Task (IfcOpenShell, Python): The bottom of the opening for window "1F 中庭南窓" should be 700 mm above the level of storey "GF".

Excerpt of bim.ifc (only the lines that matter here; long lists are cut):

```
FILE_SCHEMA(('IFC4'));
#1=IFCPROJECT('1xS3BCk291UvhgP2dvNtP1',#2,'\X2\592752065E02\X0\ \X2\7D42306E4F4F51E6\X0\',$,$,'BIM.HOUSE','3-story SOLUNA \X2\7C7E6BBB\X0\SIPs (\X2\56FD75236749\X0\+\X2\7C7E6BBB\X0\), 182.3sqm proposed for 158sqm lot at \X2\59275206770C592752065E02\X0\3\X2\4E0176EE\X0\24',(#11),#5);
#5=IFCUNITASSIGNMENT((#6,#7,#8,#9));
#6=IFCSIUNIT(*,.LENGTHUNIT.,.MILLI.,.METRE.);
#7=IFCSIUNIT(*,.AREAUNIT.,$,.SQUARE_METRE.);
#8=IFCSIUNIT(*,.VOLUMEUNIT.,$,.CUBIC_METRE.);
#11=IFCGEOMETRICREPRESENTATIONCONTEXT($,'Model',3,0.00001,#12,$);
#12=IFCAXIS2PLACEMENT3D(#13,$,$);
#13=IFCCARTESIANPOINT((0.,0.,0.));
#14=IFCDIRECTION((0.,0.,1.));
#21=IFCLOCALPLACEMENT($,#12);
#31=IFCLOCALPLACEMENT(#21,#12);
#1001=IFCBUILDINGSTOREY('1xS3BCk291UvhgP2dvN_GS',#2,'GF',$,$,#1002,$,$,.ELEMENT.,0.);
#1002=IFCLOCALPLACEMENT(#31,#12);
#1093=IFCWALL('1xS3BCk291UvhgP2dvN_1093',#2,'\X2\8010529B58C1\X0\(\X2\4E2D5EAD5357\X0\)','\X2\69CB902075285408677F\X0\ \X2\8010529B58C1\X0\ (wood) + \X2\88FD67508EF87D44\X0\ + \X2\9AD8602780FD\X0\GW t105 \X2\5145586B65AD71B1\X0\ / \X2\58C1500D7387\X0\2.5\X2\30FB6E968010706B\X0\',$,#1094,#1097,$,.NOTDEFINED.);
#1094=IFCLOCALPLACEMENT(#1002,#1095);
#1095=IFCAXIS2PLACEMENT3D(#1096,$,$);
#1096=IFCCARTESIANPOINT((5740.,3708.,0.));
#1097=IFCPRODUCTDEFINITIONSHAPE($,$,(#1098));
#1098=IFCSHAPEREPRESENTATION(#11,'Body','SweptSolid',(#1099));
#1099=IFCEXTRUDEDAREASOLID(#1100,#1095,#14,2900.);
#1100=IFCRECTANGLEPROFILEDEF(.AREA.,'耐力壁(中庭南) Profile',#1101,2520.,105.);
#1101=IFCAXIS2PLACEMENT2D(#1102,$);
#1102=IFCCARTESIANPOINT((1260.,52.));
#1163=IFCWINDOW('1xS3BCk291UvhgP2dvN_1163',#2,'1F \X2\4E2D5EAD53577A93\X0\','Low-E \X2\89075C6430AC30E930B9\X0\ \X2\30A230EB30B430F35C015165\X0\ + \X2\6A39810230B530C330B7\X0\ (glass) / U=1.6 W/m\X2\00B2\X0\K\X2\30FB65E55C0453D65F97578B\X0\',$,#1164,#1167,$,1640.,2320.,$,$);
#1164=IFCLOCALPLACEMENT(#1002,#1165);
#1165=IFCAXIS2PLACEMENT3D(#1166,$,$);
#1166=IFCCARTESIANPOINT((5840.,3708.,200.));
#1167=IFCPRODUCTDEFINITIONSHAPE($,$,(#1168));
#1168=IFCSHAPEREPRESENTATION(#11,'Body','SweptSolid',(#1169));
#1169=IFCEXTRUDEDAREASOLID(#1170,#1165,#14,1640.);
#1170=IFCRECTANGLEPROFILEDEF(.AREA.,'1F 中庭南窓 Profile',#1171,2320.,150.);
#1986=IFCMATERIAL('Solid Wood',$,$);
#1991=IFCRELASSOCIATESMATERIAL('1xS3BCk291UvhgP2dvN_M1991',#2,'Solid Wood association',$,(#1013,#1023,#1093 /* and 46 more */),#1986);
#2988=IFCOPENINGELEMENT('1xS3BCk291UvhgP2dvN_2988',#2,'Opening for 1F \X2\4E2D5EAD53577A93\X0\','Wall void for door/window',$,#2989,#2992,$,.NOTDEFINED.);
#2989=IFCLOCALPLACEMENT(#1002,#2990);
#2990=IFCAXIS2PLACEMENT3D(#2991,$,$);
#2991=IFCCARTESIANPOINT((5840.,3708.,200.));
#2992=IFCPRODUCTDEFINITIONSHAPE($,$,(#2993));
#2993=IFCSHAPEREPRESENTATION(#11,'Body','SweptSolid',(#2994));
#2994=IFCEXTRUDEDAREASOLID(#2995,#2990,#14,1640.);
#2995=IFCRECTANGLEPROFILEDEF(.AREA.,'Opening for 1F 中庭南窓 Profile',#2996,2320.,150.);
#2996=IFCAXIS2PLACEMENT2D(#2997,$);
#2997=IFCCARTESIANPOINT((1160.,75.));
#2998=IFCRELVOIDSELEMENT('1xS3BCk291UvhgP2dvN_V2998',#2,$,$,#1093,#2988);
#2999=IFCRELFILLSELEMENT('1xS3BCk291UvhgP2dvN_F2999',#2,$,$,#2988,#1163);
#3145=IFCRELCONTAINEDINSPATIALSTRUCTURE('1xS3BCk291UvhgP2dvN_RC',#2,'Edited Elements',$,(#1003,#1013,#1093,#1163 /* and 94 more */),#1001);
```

```python
import numpy as np
import ifcopenshell
import ifcopenshell.api.geometry
import ifcopenshell.geom
import ifcopenshell.util.element
import ifcopenshell.util.placement
import ifcopenshell.util.shape
import ifcopenshell.util.unit

model = ifcopenshell.open("bim.ifc")
unit_scale = ifcopenshell.util.unit.calculate_unit_scale(model)

window = model.by_id(1163)
opening = window.FillsVoids[0].RelatingOpeningElement
storey = ifcopenshell.util.element.get_container(window, ifc_class="IfcBuildingStorey")
level = ifcopenshell.util.placement.get_local_placement(storey.ObjectPlacement)[2, 3]

# The opening's origin need not be at the sill, so measure its lowest point.
shape = ifcopenshell.geom.create_shape(ifcopenshell.geom.settings(), opening)
bottom = ifcopenshell.util.shape.get_shape_bottom_elevation(shape, shape.geometry) / unit_scale
dz = level + 0.7 / unit_scale - bottom

shift = np.array([0.0, 0.0, dz])
# The window is not placed relative to its opening, so move both.
for product in (opening, window):
    matrix = ifcopenshell.util.placement.get_local_placement(product.ObjectPlacement)
    matrix[:3, 3] += shift
    ifcopenshell.api.geometry.edit_object_placement(model, product=product, matrix=matrix, is_si=False)

print(f"moved by {dz * unit_scale:+.3f} m")

model.write("bim_rev.ifc")
```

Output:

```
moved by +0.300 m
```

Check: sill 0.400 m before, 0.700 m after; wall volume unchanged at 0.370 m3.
